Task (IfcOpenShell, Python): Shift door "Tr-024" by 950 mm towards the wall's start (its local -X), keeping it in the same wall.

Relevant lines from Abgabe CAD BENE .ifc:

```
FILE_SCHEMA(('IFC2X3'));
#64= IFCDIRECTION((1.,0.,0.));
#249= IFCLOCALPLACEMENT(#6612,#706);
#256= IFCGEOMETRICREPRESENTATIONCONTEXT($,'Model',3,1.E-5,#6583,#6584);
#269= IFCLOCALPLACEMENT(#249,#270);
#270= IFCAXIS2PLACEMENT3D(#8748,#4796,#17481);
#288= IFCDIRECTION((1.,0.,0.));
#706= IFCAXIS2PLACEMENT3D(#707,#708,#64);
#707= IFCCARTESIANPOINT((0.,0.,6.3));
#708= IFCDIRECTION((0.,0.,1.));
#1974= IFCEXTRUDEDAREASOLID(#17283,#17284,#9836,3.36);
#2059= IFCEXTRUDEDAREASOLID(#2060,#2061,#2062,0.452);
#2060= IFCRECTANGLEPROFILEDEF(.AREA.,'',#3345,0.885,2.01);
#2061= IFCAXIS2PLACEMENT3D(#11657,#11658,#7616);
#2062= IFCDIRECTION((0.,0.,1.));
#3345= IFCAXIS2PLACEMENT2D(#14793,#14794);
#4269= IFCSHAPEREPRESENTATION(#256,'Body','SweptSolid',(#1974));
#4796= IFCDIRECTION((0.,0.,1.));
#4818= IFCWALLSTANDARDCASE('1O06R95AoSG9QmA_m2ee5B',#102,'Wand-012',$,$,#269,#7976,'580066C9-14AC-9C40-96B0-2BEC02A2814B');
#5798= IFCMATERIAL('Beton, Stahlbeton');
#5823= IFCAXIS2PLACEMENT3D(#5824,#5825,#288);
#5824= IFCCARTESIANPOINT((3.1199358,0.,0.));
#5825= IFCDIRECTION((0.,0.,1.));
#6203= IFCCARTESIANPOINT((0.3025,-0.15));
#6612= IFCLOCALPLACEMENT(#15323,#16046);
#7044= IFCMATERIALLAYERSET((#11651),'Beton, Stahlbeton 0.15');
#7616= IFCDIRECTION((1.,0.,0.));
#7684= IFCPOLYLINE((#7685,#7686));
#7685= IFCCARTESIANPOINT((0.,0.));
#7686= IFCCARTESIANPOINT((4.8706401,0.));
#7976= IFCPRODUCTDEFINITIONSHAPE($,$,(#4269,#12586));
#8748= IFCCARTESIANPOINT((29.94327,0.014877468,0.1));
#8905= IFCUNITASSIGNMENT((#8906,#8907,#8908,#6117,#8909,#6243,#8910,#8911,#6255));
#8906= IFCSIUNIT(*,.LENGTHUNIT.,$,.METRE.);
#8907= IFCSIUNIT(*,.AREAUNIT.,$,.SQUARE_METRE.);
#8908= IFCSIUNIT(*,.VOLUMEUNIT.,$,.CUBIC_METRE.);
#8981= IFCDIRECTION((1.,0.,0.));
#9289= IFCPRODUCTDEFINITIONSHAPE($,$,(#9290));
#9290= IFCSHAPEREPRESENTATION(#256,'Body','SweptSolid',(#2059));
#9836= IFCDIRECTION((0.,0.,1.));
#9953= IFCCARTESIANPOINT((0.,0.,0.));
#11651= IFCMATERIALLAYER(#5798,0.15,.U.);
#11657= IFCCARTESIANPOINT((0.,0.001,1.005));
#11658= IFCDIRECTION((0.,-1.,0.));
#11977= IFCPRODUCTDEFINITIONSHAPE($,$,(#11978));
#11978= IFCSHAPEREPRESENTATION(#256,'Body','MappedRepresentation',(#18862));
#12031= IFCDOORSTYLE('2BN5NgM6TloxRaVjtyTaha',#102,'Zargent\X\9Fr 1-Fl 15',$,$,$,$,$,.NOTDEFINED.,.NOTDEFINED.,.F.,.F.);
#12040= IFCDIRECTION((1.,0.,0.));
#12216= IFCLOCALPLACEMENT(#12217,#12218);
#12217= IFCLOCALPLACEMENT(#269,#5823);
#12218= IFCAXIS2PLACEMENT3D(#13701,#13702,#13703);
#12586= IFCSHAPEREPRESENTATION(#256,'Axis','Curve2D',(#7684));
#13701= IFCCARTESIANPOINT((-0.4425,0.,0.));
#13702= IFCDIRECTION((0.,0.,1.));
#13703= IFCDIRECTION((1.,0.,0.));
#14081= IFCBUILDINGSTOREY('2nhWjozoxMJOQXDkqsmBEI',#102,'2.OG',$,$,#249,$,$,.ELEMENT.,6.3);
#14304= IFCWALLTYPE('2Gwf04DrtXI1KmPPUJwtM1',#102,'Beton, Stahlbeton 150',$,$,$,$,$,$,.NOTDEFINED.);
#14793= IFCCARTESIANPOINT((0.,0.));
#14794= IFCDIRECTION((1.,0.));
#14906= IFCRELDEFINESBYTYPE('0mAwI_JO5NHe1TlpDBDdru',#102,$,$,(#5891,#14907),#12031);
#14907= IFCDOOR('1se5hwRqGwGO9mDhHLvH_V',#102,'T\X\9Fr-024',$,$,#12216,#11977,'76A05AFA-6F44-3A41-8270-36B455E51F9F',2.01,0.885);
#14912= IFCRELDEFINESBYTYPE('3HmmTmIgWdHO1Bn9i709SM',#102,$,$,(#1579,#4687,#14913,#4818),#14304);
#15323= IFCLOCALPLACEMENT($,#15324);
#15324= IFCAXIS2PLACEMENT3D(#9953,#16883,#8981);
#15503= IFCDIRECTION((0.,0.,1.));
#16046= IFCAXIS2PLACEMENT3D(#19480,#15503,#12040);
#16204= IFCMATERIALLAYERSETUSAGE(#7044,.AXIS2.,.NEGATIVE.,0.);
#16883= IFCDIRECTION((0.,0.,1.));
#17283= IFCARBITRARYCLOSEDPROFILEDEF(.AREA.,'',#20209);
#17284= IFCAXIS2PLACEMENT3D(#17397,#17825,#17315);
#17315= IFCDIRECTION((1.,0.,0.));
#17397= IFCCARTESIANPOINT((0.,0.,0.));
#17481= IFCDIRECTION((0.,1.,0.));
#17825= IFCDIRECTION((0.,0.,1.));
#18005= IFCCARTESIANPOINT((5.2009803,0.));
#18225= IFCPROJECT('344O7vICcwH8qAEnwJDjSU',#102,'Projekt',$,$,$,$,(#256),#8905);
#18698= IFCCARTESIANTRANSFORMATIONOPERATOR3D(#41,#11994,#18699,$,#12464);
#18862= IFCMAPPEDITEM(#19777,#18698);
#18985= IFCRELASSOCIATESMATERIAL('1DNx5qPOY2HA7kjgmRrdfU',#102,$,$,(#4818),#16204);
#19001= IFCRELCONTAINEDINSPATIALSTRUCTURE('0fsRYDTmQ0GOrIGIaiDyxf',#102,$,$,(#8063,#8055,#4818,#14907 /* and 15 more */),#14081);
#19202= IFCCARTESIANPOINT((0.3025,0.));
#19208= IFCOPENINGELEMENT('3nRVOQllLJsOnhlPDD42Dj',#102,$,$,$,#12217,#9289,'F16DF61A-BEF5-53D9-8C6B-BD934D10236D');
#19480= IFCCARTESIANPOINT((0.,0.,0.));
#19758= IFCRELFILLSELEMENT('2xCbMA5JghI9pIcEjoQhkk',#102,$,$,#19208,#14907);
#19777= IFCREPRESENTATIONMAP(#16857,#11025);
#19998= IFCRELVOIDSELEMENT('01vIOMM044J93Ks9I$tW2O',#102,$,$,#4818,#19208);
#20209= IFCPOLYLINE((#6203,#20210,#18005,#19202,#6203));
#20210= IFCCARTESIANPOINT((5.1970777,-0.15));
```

```python
import ifcopenshell
import ifcopenshell.api.geometry
import ifcopenshell.util.placement
import ifcopenshell.util.unit

model = ifcopenshell.open("Abgabe CAD BENE .ifc")
unit_scale = ifcopenshell.util.unit.calculate_unit_scale(model)

door = model.by_guid("1se5hwRqGwGO9mDhHLvH_V")
opening = door.FillsVoids[0].RelatingOpeningElement
wall = opening.VoidsElements[0].RelatingBuildingElement

wall_matrix = ifcopenshell.util.placement.get_local_placement(wall.ObjectPlacement)
shift = wall_matrix[:3, 0] * -0.95 / unit_scale
before = ifcopenshell.util.placement.get_local_placement(door.ObjectPlacement)[:3, 3].copy()

# The door is placed relative to its opening, so it follows when the opening moves.
matrix = ifcopenshell.util.placement.get_local_placement(opening.ObjectPlacement)
matrix[:3, 3] += shift
ifcopenshell.api.geometry.edit_object_placement(
    model, product=opening, matrix=matrix, is_si=False, should_transform_children=True
)

after = ifcopenshell.util.placement.get_local_placement(door.ObjectPlacement)[:3, 3]
print("door moved by", (after - before).round(3) + 0.0)

model.write("Abgabe CAD BENE _v2.ifc")
```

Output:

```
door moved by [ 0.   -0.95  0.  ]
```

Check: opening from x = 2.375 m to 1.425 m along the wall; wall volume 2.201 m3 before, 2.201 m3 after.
